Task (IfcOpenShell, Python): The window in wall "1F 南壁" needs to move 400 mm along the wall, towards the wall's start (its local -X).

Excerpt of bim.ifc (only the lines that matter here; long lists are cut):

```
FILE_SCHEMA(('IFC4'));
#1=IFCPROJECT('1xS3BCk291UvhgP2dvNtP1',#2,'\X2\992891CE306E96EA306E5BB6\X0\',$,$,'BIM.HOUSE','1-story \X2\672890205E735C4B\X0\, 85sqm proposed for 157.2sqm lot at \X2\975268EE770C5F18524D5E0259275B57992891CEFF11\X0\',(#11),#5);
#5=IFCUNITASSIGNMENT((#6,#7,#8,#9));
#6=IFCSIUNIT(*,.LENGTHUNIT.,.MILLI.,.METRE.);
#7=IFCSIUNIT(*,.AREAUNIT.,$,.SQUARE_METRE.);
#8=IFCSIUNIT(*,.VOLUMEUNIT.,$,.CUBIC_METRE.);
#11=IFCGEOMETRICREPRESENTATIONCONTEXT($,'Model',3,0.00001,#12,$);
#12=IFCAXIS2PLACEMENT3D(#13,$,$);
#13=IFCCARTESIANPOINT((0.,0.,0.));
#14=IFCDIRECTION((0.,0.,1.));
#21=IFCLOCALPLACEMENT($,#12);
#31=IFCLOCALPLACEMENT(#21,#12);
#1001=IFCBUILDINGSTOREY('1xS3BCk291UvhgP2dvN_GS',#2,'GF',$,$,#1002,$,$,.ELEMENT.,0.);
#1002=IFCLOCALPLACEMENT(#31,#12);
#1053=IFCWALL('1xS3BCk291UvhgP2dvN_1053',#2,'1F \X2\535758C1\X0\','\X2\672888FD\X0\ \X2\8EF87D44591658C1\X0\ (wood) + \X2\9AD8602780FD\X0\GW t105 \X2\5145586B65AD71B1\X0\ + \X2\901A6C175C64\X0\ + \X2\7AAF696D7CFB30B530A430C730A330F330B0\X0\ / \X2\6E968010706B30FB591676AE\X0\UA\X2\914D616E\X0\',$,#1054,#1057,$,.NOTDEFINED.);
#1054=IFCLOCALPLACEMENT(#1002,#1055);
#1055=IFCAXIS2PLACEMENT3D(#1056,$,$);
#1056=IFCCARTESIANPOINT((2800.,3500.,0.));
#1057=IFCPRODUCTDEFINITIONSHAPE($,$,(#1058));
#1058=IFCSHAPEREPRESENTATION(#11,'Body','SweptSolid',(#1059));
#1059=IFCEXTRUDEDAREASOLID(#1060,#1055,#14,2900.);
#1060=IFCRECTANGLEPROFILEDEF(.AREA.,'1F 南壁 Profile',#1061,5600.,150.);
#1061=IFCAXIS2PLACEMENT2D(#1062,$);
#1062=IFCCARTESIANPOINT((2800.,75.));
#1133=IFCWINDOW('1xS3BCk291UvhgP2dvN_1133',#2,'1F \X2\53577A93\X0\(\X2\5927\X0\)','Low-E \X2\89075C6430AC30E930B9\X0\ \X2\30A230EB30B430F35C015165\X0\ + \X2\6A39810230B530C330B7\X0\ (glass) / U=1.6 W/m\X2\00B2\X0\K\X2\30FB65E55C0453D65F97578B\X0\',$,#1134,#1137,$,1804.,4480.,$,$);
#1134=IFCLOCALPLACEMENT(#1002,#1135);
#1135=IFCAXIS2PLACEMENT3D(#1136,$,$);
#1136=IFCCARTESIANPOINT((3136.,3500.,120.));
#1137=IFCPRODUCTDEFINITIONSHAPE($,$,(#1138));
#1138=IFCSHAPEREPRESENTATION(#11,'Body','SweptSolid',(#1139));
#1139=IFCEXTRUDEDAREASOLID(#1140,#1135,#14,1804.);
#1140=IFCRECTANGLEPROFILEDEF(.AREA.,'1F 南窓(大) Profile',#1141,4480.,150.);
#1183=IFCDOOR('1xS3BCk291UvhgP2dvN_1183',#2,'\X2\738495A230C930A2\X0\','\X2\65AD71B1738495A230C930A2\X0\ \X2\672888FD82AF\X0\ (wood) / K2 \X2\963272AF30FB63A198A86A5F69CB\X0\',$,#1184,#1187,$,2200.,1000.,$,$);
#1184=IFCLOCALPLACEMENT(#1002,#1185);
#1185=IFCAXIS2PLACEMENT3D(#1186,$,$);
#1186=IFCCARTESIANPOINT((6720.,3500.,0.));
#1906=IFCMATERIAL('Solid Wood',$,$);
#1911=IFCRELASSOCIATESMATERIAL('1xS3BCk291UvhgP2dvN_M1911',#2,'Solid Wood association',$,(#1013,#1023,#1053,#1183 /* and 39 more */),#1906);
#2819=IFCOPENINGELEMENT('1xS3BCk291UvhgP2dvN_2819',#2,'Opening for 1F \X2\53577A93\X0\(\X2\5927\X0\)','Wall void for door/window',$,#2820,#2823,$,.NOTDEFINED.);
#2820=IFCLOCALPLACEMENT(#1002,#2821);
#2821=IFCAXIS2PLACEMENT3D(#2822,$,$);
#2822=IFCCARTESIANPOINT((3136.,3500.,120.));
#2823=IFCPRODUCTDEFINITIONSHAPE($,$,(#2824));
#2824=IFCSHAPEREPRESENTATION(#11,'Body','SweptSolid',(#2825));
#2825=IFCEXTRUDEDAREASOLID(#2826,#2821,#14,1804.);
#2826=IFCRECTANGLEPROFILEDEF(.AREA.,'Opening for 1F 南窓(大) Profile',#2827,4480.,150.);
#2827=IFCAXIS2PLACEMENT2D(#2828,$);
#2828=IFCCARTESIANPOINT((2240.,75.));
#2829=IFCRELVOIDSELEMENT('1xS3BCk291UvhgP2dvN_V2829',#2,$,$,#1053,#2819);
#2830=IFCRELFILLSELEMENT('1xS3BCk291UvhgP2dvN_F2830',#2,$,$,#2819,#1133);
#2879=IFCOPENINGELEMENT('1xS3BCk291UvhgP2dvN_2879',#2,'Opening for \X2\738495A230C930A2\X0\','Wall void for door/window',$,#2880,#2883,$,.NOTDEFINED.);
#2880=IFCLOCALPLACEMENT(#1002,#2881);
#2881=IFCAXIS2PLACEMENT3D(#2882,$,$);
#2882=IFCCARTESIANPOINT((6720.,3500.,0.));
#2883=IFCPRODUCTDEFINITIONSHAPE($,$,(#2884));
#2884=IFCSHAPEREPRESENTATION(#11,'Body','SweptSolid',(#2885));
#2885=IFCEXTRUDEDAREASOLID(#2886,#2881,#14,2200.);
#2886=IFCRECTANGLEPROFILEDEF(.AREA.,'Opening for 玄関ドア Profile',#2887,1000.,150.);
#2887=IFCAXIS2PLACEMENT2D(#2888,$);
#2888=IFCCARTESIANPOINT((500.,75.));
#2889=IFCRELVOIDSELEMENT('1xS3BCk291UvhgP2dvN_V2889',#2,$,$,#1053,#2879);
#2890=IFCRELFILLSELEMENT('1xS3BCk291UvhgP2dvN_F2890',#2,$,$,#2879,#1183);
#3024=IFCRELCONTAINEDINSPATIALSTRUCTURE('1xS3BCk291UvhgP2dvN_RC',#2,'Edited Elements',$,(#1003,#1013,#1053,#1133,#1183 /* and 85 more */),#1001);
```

```python
import ifcopenshell
import ifcopenshell.api.geometry
import ifcopenshell.util.placement
import ifcopenshell.util.unit

model = ifcopenshell.open("bim.ifc")
unit_scale = ifcopenshell.util.unit.calculate_unit_scale(model)

window = model.by_id(1133)
opening = window.FillsVoids[0].RelatingOpeningElement
wall = opening.VoidsElements[0].RelatingBuildingElement

wall_matrix = ifcopenshell.util.placement.get_local_placement(wall.ObjectPlacement)
shift = wall_matrix[:3, 0] * -0.4 / unit_scale
before = ifcopenshell.util.placement.get_local_placement(window.ObjectPlacement)[:3, 3].copy()

# The window is not placed relative to its opening, so move both.
for product in (opening, window):
    matrix = ifcopenshell.util.placement.get_local_placement(product.ObjectPlacement)
    matrix[:3, 3] += shift
    ifcopenshell.api.geometry.edit_object_placement(model, product=product, matrix=matrix, is_si=False)

after = ifcopenshell.util.placement.get_local_placement(window.ObjectPlacement)[:3, 3]
print("window moved by", (after - before).round(3) + 0.0)

model.write("bim_updated.ifc")
```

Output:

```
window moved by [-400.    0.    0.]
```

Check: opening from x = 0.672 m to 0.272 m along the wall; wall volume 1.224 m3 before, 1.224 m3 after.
